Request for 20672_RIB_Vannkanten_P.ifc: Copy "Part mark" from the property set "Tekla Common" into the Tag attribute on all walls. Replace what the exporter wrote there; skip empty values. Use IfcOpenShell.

First a look at what the model holds.

```python
import ifcopenshell
import ifcopenshell.util.element

model = ifcopenshell.open("20672_RIB_Vannkanten_P.ifc")
print(model.schema)
walls = model.by_type("IfcWall")
print(len(walls), "walls")
for e in walls[:8]:
    source = ifcopenshell.util.element.get_pset(e, "Tekla Common", "Part mark")
    target = e.Tag
    print(e.id(), repr(source), repr(target), sep=" | ")
```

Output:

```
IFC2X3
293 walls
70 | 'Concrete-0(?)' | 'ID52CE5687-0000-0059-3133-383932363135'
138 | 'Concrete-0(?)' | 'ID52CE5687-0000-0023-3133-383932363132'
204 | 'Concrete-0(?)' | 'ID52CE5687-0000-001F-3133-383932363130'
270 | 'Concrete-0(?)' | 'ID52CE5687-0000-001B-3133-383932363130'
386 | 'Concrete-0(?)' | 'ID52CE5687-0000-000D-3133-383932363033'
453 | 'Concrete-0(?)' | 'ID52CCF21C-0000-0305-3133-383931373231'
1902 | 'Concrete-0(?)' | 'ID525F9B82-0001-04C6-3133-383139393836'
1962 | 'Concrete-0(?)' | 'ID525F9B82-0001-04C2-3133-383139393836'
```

```python
import ifcopenshell
import ifcopenshell.util.element

model = ifcopenshell.open("20672_RIB_Vannkanten_P.ifc")

count = 0
for e in model.by_type("IfcWall"):
    value = ifcopenshell.util.element.get_pset(e, "Tekla Common", "Part mark")
    current = e.Tag
    if not value or not value.strip() or current == value:
        continue
    e.Tag = value
    count += 1

print(count, "walls updated")

model.write("20672_RIB_Vannkanten_P_edited.ifc")
```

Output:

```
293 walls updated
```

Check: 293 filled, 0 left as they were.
